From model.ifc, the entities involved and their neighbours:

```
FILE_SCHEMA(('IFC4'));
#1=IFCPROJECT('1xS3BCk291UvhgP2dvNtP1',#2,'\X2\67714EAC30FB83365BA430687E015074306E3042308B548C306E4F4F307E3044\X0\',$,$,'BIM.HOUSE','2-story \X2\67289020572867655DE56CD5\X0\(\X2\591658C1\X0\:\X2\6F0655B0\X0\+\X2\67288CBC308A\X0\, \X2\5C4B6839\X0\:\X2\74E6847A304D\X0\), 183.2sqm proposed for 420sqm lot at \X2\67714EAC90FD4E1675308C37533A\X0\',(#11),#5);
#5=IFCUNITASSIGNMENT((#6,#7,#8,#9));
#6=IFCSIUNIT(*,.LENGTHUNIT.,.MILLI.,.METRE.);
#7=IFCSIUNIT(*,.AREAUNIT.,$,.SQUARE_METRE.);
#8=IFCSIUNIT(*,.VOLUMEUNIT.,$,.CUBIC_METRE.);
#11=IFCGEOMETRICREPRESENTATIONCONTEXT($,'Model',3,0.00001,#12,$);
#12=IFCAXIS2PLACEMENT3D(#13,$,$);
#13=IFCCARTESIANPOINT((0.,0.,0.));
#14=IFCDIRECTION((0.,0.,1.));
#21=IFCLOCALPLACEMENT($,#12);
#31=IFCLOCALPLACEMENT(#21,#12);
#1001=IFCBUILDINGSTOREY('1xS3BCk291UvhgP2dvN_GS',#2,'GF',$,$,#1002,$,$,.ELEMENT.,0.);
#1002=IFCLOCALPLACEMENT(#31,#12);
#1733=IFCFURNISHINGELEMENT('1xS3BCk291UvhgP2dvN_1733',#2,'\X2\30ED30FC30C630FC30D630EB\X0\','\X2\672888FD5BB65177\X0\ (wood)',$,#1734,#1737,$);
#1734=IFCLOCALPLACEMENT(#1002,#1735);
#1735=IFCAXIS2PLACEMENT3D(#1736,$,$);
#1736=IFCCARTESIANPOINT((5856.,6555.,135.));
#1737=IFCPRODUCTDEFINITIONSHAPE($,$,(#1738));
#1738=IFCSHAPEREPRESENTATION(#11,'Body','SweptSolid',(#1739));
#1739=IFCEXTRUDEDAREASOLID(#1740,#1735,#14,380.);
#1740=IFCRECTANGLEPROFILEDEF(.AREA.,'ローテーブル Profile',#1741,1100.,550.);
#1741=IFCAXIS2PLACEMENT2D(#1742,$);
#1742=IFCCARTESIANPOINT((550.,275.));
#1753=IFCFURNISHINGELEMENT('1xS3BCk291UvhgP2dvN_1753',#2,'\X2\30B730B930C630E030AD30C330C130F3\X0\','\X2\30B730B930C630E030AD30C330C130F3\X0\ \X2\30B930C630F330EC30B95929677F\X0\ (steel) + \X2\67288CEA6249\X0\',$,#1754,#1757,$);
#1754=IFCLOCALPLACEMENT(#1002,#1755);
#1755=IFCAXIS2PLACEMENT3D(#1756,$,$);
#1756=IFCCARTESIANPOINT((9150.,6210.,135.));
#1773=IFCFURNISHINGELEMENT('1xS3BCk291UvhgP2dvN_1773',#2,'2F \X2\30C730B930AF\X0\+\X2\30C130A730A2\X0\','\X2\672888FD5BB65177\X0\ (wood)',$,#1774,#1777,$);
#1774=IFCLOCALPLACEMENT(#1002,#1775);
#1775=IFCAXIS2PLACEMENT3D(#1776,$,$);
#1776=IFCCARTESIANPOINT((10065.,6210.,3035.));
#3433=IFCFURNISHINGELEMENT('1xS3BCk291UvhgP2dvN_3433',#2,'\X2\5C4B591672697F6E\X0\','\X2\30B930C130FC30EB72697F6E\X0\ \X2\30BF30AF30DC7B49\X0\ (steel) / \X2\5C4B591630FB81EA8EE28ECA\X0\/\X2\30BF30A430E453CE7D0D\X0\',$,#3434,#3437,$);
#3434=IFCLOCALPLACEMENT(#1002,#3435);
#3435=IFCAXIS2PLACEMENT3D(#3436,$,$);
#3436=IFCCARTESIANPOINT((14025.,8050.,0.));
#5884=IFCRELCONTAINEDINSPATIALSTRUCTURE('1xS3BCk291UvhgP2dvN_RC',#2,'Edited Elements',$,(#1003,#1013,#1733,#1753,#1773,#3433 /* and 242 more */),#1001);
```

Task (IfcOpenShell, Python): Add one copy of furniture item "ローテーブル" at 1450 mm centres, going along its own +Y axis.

```python
import ifcopenshell
import ifcopenshell.api.geometry
import ifcopenshell.api.root
import ifcopenshell.util.element
import ifcopenshell.util.placement
import ifcopenshell.util.unit

model = ifcopenshell.open("model.ifc")
unit_scale = ifcopenshell.util.unit.calculate_unit_scale(model)


def reuse_history(source, copy):
    """copy_class also copies each property set's owner history, people and application; keep the originals."""
    for rel in copy.IsDefinedBy:
        if rel.is_a("IfcRelDefinesByProperties") and (history := rel.RelatingPropertyDefinition.OwnerHistory):
            rel.RelatingPropertyDefinition.OwnerHistory = source.OwnerHistory
            ifcopenshell.util.element.remove_deep2(model, history)


source = model.by_id(1733)
base = ifcopenshell.util.placement.get_local_placement(source.ObjectPlacement)
step = base[:3, 1] * 1.45 / unit_scale

for i in range(1, 2):
    copy = ifcopenshell.api.root.copy_class(model, product=source)
    copy.Representation = ifcopenshell.util.element.copy_deep(
        model, source.Representation, exclude=["IfcGeometricRepresentationContext", "IfcRepresentationMap"]
    )
    reuse_history(source, copy)
    matrix = base.copy()
    matrix[:3, 3] += i * step
    print("added at", matrix[:3, 3].round(3) + 0.0)
    ifcopenshell.api.geometry.edit_object_placement(model, product=copy, matrix=matrix, is_si=False)

model.write("model-out.ifc")
```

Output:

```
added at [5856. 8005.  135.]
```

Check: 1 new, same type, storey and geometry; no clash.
